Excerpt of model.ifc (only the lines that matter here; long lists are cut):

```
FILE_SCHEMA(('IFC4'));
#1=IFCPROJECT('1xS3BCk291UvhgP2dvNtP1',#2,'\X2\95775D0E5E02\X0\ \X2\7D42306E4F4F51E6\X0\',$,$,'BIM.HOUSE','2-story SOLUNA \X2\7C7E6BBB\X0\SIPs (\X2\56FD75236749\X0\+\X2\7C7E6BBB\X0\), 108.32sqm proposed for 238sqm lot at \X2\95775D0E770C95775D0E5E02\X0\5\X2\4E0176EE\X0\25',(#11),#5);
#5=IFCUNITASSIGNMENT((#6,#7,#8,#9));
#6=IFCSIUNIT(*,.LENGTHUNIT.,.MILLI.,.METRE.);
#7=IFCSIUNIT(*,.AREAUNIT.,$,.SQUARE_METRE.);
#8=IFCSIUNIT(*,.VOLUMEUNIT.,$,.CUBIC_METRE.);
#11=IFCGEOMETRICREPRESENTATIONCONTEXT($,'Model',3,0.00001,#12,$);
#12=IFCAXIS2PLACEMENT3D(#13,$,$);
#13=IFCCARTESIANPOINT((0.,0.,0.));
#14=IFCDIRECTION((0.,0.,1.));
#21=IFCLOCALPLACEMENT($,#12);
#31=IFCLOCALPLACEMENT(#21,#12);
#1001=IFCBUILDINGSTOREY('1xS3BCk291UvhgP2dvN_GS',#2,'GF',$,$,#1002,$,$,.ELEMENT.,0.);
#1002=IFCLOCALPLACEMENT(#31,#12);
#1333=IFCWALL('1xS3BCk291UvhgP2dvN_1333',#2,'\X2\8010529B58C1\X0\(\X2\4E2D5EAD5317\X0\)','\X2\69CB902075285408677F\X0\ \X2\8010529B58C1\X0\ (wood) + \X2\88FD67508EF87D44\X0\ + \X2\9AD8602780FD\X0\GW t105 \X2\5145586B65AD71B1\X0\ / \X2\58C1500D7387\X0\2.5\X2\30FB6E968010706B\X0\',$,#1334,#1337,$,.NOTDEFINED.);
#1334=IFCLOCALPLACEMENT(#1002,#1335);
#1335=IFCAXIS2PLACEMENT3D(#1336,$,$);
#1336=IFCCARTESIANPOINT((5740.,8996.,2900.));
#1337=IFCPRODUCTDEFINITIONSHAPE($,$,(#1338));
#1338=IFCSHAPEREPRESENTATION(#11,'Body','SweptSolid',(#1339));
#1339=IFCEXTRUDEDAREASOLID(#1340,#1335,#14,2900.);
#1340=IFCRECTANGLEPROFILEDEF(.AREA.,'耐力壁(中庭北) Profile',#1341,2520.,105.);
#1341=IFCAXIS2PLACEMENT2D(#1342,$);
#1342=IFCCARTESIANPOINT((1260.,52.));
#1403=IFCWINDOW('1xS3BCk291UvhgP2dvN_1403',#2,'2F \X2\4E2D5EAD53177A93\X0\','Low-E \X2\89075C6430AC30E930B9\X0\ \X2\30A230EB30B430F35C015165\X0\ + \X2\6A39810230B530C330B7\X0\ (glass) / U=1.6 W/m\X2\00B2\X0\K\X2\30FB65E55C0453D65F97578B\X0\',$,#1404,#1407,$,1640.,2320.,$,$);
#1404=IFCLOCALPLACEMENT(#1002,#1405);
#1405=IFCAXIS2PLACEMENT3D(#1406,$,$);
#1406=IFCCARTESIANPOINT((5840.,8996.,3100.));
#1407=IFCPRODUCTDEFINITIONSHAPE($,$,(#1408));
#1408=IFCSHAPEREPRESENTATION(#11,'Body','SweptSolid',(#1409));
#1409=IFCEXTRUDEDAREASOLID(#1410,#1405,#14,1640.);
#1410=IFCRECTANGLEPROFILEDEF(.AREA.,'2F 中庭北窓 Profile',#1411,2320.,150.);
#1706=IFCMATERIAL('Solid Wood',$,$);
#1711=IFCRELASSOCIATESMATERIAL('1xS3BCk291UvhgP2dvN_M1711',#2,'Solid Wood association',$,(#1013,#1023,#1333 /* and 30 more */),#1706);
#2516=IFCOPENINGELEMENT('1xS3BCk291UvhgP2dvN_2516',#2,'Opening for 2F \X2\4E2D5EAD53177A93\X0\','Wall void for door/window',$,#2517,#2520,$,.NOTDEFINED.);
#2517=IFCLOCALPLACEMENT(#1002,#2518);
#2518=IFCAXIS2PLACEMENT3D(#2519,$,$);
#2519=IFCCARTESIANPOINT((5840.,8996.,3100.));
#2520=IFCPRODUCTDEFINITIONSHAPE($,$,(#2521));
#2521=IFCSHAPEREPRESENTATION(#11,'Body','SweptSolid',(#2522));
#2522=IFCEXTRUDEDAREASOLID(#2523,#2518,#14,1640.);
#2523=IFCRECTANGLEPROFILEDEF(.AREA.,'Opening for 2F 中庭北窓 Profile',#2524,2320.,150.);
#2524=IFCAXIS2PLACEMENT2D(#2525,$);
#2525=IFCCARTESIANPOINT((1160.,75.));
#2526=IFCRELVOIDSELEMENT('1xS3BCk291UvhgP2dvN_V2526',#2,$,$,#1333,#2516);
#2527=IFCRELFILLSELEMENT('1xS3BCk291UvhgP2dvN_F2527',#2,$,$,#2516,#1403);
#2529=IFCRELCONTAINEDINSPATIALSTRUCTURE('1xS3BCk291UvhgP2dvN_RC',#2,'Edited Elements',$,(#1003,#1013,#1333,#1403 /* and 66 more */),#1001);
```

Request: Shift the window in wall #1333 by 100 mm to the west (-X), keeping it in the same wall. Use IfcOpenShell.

```python
import ifcopenshell
import ifcopenshell.api.geometry
import ifcopenshell.util.placement
import ifcopenshell.util.unit

model = ifcopenshell.open("model.ifc")
unit_scale = ifcopenshell.util.unit.calculate_unit_scale(model)

window = model.by_id(1403)
opening = window.FillsVoids[0].RelatingOpeningElement
wall = opening.VoidsElements[0].RelatingBuildingElement

wall_matrix = ifcopenshell.util.placement.get_local_placement(wall.ObjectPlacement)
shift = wall_matrix[:3, 0] * -0.1 / unit_scale
before = ifcopenshell.util.placement.get_local_placement(window.ObjectPlacement)[:3, 3].copy()

# The window is not placed relative to its opening, so move both.
for product in (opening, window):
    matrix = ifcopenshell.util.placement.get_local_placement(product.ObjectPlacement)
    matrix[:3, 3] += shift
    ifcopenshell.api.geometry.edit_object_placement(model, product=product, matrix=matrix, is_si=False)

after = ifcopenshell.util.placement.get_local_placement(window.ObjectPlacement)[:3, 3]
print("window moved by", (after - before).round(3) + 0.0)

model.write("model_v2.ifc")
```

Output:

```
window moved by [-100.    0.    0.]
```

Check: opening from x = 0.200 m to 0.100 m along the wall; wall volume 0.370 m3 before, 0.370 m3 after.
